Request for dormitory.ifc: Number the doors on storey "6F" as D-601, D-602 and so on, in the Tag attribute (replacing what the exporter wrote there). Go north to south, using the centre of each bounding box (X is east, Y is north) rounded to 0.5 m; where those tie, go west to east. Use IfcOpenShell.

First a look at what the model holds.

```python
import ifcopenshell
import ifcopenshell.util.element
import ifcopenshell.util.placement

model = ifcopenshell.open("dormitory.ifc")
print(model.schema)
storey = next(s for s in model.by_type("IfcBuildingStorey") if s.Name == "6F")
doors = [e for e in ifcopenshell.util.element.get_decomposition(storey) if e.is_a("IfcDoor")]
for e in sorted(doors, key=lambda e: e.id()):
    origin = ifcopenshell.util.placement.get_local_placement(e.ObjectPlacement)[:3, 3]
    print(e.id(), e.Tag, e.Name, origin.round(2) + 0.0, sep=" | ")
```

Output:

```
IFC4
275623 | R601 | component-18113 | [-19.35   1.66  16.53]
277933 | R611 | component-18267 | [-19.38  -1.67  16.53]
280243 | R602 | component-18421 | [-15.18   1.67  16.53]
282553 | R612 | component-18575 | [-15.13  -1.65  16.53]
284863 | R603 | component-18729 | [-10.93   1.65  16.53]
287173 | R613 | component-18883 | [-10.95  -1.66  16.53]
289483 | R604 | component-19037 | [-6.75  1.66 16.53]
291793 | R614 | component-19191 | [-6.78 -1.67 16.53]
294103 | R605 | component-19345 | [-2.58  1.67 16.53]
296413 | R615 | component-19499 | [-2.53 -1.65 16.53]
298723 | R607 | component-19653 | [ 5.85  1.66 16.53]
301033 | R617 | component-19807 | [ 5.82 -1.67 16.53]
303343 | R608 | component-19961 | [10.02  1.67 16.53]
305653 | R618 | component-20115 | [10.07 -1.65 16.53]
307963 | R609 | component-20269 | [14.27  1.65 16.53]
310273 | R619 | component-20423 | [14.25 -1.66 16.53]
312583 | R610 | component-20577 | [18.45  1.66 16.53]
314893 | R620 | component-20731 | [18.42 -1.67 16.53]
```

```python
import ifcopenshell
import ifcopenshell.geom
import ifcopenshell.util.element
import ifcopenshell.util.shape

model = ifcopenshell.open("dormitory.ifc")
settings = ifcopenshell.geom.settings()
settings.set("use-world-coords", True)


def centre(element):
    shape = ifcopenshell.geom.create_shape(settings, element)
    return ifcopenshell.util.shape.get_bbox_centroid(shape.geometry)


storey = next(s for s in model.by_type("IfcBuildingStorey") if s.Name == "6F")
doors = [e for e in ifcopenshell.util.element.get_decomposition(storey) if e.is_a("IfcDoor")]

# Insertion points can sit at a corner or the storey origin, so sort by the geometry (in metres).
centres = {e: centre(e) for e in doors}
doors.sort(key=lambda e: (-round(centres[e][1] / 0.5), centres[e][0]))

for i, e in enumerate(doors, start=1):
    number = f"D-6{i:02d}"
    e.Tag = number
    print(e.id(), number)

model.write("dormitory_updated.ifc")
```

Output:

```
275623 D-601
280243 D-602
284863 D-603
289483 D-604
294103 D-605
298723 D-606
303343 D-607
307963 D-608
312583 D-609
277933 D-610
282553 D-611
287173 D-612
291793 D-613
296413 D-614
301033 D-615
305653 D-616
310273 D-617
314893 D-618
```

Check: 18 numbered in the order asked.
